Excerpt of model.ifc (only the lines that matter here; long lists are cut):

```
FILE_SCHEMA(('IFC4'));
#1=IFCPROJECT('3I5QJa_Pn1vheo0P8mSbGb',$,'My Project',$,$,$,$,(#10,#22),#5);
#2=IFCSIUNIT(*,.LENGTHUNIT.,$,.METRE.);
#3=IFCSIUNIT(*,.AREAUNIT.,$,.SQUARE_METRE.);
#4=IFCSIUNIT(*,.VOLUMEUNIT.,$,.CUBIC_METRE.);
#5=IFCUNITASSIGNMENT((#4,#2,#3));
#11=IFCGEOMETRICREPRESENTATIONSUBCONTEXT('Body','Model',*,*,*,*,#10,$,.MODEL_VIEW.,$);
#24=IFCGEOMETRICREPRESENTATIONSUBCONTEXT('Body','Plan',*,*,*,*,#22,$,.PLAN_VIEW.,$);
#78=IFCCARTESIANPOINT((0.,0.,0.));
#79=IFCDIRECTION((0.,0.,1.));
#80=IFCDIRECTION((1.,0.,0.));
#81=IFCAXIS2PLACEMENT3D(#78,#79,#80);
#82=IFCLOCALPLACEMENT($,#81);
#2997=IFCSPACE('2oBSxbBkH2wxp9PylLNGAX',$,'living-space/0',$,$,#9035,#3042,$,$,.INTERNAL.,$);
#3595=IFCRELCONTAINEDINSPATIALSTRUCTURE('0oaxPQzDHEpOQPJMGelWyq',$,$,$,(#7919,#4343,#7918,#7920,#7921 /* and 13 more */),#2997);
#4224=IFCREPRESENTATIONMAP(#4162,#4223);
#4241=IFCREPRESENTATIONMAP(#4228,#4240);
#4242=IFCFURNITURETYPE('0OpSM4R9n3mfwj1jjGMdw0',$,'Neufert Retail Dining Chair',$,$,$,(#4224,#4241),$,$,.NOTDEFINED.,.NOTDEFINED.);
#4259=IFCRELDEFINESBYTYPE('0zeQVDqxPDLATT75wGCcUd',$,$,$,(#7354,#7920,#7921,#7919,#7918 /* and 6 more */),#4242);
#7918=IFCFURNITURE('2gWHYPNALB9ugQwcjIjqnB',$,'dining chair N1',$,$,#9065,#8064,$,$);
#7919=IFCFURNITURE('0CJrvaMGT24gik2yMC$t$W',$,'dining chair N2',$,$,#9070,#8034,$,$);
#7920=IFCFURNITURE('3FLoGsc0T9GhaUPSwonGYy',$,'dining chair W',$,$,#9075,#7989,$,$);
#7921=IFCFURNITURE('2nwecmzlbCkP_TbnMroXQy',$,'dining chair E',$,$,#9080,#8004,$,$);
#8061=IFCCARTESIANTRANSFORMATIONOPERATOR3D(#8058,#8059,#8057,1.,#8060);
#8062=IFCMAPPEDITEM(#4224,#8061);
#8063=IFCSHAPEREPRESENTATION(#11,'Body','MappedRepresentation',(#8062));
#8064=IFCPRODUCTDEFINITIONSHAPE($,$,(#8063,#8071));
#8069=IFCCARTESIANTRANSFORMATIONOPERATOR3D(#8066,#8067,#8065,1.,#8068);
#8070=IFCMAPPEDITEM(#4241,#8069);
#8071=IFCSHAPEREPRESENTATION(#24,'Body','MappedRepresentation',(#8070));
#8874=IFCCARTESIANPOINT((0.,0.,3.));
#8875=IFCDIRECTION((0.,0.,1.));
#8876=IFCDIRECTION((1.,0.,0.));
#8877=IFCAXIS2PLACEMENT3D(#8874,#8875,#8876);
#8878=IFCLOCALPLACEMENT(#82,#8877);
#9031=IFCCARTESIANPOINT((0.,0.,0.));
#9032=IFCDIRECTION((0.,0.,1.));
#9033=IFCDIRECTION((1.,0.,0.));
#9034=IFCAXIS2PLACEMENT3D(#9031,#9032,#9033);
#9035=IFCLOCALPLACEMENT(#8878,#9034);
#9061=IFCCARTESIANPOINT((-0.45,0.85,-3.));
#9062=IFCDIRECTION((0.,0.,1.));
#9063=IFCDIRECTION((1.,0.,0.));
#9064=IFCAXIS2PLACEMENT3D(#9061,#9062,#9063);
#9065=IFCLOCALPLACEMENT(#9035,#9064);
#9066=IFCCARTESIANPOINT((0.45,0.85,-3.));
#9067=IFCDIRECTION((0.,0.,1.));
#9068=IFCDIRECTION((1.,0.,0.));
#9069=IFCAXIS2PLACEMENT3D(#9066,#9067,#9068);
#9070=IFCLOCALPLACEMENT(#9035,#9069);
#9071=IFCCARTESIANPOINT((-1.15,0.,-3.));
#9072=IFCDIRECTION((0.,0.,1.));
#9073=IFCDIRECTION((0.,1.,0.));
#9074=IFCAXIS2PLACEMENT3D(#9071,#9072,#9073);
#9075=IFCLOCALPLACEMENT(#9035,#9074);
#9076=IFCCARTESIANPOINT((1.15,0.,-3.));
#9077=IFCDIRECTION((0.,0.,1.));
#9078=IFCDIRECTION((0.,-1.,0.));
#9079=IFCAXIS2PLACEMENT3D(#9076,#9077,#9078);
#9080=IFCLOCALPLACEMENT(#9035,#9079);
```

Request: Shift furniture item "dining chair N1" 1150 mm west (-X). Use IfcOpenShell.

```python
import ifcopenshell
import ifcopenshell.api.geometry
import ifcopenshell.util.placement
import ifcopenshell.util.unit

model = ifcopenshell.open("model.ifc")
unit_scale = ifcopenshell.util.unit.calculate_unit_scale(model)

item = model.by_id(7918)
matrix = ifcopenshell.util.placement.get_local_placement(item.ObjectPlacement)
matrix[0, 3] -= 1.15 / unit_scale
ifcopenshell.api.geometry.edit_object_placement(model, product=item, matrix=matrix, is_si=False)

print(ifcopenshell.util.placement.get_local_placement(item.ObjectPlacement).round(3) + 0.0)

model.write("model_v2.ifc")
```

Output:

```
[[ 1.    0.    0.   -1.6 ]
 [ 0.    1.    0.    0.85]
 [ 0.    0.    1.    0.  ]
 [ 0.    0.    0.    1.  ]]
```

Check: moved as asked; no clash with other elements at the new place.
